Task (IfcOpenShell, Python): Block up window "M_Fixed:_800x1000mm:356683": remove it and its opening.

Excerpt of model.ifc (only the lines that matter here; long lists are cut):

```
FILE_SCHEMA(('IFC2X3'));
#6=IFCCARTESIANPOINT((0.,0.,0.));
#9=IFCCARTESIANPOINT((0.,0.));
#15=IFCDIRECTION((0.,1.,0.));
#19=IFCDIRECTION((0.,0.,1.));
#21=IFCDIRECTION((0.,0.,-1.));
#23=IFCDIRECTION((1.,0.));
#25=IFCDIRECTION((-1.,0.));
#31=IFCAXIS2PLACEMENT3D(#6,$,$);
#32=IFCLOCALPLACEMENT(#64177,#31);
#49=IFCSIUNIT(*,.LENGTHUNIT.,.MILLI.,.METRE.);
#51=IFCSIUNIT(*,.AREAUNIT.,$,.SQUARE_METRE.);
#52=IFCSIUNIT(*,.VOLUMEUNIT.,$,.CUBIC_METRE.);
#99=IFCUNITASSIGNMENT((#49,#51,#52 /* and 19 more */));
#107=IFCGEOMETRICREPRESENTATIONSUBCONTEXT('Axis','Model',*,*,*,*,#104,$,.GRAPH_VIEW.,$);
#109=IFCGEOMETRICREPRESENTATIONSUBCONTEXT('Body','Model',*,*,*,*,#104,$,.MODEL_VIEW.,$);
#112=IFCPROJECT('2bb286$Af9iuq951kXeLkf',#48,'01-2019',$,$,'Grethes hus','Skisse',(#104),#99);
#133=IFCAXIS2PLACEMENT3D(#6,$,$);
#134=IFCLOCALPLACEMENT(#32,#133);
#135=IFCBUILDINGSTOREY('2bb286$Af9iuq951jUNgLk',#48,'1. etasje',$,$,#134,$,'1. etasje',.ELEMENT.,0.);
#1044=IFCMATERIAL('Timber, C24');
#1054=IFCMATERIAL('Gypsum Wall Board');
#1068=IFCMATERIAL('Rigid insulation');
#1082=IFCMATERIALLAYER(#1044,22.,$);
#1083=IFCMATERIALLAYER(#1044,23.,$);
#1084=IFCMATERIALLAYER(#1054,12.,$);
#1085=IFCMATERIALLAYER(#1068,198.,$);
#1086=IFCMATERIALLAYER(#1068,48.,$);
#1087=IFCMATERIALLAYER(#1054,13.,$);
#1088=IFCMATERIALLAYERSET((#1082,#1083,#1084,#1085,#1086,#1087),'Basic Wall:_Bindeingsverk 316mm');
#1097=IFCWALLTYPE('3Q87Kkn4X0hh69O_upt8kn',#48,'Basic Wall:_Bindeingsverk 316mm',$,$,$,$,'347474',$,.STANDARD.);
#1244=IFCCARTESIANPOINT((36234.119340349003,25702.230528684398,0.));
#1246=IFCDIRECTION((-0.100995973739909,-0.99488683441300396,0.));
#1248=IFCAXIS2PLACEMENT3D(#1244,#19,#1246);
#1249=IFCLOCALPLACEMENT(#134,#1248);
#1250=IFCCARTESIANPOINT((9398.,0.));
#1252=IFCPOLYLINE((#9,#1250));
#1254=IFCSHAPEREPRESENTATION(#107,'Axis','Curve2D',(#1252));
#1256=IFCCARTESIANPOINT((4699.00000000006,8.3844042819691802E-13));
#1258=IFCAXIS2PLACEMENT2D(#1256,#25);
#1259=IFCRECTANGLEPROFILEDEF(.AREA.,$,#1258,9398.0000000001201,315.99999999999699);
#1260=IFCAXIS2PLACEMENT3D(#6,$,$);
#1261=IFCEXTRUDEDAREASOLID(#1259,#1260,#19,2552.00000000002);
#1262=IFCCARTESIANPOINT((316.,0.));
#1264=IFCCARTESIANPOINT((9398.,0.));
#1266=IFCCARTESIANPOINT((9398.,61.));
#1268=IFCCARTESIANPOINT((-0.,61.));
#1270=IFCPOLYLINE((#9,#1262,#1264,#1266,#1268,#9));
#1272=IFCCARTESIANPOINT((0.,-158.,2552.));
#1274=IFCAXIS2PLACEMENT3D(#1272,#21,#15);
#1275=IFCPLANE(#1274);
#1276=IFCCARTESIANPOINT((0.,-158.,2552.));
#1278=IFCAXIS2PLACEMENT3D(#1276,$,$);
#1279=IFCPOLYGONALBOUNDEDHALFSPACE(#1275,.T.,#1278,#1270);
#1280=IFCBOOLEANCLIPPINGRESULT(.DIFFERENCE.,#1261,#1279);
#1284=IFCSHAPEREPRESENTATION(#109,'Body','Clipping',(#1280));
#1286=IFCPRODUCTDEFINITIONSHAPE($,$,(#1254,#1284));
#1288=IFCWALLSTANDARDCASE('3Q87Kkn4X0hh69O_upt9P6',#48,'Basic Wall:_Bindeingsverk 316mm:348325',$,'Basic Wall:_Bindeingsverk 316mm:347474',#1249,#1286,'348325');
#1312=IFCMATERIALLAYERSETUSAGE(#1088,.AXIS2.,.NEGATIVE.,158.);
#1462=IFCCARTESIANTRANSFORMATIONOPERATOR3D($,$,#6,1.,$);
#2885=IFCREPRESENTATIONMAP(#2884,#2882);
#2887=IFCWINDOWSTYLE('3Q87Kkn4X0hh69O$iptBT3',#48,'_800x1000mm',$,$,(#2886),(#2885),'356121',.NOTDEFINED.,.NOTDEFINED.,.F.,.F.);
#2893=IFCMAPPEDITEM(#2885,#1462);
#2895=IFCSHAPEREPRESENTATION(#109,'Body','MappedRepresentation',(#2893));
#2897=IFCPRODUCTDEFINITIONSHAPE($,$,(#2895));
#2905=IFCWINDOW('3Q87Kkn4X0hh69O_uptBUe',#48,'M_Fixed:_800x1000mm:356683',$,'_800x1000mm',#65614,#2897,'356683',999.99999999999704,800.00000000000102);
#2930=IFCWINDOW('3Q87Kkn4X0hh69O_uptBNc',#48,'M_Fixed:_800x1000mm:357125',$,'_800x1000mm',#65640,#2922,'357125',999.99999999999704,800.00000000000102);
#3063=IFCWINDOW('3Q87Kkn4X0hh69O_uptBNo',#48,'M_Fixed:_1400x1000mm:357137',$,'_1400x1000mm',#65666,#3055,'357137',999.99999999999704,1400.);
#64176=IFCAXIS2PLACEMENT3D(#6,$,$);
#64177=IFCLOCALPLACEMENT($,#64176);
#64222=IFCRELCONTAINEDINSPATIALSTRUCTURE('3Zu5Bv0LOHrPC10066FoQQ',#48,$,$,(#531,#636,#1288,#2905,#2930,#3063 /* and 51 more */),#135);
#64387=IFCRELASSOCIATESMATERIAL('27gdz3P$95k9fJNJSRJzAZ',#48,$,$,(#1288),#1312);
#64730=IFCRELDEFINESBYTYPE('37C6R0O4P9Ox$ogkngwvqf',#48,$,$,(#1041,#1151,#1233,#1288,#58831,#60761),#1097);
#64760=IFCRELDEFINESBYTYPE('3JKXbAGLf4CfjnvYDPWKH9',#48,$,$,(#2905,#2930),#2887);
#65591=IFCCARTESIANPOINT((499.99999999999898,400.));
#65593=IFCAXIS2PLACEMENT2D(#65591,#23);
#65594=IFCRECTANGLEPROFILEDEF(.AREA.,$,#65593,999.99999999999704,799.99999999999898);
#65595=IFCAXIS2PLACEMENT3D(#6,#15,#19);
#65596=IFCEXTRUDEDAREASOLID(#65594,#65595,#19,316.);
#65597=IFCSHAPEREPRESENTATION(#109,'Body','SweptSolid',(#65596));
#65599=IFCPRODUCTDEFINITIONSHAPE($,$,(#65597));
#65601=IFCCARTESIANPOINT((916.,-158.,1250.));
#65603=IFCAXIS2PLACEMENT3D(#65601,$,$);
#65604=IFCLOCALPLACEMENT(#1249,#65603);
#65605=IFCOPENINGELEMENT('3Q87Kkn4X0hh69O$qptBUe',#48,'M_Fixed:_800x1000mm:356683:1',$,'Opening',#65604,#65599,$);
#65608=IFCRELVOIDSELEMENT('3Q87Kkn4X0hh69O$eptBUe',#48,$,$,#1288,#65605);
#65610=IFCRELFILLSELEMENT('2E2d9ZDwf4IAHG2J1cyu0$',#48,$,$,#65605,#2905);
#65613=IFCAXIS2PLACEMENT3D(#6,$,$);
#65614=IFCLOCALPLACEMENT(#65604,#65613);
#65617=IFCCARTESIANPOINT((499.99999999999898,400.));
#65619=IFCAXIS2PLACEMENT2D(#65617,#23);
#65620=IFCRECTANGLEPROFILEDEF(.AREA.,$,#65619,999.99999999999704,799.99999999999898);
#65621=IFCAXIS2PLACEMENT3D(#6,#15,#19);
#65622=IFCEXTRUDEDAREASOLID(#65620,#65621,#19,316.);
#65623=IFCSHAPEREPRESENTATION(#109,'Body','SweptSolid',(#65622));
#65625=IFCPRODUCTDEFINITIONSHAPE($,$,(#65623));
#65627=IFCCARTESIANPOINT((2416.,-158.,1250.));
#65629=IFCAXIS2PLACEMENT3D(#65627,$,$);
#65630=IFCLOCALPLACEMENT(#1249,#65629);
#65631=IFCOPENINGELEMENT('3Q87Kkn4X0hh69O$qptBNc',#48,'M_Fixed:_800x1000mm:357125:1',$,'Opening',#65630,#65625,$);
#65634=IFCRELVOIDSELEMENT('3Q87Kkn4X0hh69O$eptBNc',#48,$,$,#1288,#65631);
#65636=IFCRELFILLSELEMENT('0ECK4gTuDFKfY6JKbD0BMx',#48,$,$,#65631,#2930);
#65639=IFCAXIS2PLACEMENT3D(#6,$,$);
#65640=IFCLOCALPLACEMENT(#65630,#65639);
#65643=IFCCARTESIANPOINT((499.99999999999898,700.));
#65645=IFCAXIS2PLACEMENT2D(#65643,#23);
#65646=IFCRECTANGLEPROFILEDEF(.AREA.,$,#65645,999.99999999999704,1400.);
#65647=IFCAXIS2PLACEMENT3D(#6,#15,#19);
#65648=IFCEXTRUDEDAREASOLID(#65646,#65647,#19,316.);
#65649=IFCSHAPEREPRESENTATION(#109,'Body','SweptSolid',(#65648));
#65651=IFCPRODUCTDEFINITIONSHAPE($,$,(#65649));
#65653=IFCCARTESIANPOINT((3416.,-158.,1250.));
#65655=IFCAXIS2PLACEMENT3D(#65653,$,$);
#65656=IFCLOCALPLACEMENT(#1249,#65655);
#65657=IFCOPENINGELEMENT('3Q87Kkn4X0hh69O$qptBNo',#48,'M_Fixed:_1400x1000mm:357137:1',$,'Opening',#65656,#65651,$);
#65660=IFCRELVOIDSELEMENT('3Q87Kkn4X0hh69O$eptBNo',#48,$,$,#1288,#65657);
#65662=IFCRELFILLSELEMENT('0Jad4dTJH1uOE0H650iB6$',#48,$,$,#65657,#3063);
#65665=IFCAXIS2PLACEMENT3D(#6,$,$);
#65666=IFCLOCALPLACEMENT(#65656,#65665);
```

```python
import ifcopenshell
import ifcopenshell.api.feature
import ifcopenshell.api.root
import ifcopenshell.geom
import ifcopenshell.util.shape

model = ifcopenshell.open("model.ifc")
settings = ifcopenshell.geom.settings()


def volume(element):
    """Net volume in cubic metres, openings subtracted."""
    shape = ifcopenshell.geom.create_shape(settings, element)
    return ifcopenshell.util.shape.get_volume(shape.geometry)


window = model.by_guid("3Q87Kkn4X0hh69O_uptBUe")
opening = window.FillsVoids[0].RelatingOpeningElement
wall = opening.VoidsElements[0].RelatingBuildingElement
before = volume(wall)

ifcopenshell.api.root.remove_product(model, product=window)
ifcopenshell.api.feature.remove_feature(model, feature=opening)

after = volume(wall)

print(f"wall volume {before:.3f} -> {after:.3f} m3")

model.write("model_edited.ifc")
```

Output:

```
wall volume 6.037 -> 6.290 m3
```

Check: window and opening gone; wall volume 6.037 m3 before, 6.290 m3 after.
